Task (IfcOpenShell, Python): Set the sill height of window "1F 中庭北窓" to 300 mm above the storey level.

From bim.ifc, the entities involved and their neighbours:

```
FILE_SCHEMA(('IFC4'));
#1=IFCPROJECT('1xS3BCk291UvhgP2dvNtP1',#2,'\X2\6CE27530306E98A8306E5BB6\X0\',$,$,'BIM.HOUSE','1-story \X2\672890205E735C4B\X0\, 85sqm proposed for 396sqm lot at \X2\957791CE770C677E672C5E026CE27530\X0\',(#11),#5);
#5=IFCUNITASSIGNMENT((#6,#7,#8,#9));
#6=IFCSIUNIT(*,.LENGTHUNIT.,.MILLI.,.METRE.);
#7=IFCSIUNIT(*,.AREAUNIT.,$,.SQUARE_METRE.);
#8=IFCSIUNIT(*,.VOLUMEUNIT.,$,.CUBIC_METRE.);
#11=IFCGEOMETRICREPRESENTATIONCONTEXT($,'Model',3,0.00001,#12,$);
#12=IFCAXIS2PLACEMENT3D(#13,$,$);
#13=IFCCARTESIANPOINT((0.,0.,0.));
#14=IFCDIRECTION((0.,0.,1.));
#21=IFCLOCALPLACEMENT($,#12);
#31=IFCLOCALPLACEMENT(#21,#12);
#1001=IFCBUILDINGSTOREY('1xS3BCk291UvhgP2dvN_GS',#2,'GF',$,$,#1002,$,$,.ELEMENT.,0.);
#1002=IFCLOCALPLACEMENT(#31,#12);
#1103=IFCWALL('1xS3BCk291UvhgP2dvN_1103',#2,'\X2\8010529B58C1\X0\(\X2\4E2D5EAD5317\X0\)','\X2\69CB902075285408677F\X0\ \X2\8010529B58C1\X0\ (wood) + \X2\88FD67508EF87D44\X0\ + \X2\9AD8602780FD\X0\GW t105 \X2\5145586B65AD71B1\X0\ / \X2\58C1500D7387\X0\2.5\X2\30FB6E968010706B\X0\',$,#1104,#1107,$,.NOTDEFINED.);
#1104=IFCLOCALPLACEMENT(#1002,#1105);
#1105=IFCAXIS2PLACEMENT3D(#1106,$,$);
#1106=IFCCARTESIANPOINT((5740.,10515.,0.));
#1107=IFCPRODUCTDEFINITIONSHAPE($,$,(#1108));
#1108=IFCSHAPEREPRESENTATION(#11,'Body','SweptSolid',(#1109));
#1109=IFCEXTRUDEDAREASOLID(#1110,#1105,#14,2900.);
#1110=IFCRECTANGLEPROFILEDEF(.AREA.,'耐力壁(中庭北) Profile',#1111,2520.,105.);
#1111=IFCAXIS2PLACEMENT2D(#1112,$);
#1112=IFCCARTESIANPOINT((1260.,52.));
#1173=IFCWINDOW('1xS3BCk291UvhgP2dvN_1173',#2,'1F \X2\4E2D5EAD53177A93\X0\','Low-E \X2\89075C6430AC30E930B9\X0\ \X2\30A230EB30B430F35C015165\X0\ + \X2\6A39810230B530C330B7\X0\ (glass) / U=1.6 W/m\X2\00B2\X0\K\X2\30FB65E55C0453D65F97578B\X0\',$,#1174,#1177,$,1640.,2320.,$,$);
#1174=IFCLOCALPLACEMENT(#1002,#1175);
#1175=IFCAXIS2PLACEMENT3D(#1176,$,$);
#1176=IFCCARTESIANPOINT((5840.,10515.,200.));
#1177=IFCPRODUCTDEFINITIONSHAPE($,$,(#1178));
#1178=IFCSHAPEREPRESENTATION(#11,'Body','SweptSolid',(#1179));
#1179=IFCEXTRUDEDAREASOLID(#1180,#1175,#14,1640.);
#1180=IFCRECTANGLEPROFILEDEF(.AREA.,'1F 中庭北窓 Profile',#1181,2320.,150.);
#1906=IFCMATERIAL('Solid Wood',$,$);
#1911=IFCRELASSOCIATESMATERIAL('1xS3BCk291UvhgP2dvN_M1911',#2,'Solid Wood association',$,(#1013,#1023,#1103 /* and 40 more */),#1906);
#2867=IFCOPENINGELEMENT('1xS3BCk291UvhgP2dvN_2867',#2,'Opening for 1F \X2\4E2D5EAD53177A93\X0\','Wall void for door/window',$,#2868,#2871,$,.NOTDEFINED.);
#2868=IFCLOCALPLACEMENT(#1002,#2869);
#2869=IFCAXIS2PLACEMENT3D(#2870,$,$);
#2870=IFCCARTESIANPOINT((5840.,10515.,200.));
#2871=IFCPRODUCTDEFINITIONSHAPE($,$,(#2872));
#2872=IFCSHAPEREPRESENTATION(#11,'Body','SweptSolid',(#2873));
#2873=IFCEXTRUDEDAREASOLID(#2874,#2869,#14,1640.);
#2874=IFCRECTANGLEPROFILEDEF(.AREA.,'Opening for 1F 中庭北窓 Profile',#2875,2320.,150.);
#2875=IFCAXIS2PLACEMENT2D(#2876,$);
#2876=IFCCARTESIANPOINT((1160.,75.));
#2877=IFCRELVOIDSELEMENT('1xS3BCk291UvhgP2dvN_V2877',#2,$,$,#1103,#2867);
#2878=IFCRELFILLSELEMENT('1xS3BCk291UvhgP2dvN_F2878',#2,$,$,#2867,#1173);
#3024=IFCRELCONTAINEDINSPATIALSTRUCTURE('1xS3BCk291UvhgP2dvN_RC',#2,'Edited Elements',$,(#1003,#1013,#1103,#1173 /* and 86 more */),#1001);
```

```python
import numpy as np
import ifcopenshell
import ifcopenshell.api.geometry
import ifcopenshell.geom
import ifcopenshell.util.element
import ifcopenshell.util.placement
import ifcopenshell.util.shape
import ifcopenshell.util.unit

model = ifcopenshell.open("bim.ifc")
unit_scale = ifcopenshell.util.unit.calculate_unit_scale(model)

window = model.by_id(1173)
opening = window.FillsVoids[0].RelatingOpeningElement
storey = ifcopenshell.util.element.get_container(window, ifc_class="IfcBuildingStorey")
level = ifcopenshell.util.placement.get_local_placement(storey.ObjectPlacement)[2, 3]

# The opening's origin need not be at the sill, so measure its lowest point.
shape = ifcopenshell.geom.create_shape(ifcopenshell.geom.settings(), opening)
bottom = ifcopenshell.util.shape.get_shape_bottom_elevation(shape, shape.geometry) / unit_scale
dz = level + 0.3 / unit_scale - bottom

shift = np.array([0.0, 0.0, dz])
# The window is not placed relative to its opening, so move both.
for product in (opening, window):
    matrix = ifcopenshell.util.placement.get_local_placement(product.ObjectPlacement)
    matrix[:3, 3] += shift
    ifcopenshell.api.geometry.edit_object_placement(model, product=product, matrix=matrix, is_si=False)

print(f"moved by {dz * unit_scale:+.3f} m")

model.write("bim_updated.ifc")
```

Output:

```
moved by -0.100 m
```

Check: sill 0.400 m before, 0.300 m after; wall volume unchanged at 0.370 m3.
